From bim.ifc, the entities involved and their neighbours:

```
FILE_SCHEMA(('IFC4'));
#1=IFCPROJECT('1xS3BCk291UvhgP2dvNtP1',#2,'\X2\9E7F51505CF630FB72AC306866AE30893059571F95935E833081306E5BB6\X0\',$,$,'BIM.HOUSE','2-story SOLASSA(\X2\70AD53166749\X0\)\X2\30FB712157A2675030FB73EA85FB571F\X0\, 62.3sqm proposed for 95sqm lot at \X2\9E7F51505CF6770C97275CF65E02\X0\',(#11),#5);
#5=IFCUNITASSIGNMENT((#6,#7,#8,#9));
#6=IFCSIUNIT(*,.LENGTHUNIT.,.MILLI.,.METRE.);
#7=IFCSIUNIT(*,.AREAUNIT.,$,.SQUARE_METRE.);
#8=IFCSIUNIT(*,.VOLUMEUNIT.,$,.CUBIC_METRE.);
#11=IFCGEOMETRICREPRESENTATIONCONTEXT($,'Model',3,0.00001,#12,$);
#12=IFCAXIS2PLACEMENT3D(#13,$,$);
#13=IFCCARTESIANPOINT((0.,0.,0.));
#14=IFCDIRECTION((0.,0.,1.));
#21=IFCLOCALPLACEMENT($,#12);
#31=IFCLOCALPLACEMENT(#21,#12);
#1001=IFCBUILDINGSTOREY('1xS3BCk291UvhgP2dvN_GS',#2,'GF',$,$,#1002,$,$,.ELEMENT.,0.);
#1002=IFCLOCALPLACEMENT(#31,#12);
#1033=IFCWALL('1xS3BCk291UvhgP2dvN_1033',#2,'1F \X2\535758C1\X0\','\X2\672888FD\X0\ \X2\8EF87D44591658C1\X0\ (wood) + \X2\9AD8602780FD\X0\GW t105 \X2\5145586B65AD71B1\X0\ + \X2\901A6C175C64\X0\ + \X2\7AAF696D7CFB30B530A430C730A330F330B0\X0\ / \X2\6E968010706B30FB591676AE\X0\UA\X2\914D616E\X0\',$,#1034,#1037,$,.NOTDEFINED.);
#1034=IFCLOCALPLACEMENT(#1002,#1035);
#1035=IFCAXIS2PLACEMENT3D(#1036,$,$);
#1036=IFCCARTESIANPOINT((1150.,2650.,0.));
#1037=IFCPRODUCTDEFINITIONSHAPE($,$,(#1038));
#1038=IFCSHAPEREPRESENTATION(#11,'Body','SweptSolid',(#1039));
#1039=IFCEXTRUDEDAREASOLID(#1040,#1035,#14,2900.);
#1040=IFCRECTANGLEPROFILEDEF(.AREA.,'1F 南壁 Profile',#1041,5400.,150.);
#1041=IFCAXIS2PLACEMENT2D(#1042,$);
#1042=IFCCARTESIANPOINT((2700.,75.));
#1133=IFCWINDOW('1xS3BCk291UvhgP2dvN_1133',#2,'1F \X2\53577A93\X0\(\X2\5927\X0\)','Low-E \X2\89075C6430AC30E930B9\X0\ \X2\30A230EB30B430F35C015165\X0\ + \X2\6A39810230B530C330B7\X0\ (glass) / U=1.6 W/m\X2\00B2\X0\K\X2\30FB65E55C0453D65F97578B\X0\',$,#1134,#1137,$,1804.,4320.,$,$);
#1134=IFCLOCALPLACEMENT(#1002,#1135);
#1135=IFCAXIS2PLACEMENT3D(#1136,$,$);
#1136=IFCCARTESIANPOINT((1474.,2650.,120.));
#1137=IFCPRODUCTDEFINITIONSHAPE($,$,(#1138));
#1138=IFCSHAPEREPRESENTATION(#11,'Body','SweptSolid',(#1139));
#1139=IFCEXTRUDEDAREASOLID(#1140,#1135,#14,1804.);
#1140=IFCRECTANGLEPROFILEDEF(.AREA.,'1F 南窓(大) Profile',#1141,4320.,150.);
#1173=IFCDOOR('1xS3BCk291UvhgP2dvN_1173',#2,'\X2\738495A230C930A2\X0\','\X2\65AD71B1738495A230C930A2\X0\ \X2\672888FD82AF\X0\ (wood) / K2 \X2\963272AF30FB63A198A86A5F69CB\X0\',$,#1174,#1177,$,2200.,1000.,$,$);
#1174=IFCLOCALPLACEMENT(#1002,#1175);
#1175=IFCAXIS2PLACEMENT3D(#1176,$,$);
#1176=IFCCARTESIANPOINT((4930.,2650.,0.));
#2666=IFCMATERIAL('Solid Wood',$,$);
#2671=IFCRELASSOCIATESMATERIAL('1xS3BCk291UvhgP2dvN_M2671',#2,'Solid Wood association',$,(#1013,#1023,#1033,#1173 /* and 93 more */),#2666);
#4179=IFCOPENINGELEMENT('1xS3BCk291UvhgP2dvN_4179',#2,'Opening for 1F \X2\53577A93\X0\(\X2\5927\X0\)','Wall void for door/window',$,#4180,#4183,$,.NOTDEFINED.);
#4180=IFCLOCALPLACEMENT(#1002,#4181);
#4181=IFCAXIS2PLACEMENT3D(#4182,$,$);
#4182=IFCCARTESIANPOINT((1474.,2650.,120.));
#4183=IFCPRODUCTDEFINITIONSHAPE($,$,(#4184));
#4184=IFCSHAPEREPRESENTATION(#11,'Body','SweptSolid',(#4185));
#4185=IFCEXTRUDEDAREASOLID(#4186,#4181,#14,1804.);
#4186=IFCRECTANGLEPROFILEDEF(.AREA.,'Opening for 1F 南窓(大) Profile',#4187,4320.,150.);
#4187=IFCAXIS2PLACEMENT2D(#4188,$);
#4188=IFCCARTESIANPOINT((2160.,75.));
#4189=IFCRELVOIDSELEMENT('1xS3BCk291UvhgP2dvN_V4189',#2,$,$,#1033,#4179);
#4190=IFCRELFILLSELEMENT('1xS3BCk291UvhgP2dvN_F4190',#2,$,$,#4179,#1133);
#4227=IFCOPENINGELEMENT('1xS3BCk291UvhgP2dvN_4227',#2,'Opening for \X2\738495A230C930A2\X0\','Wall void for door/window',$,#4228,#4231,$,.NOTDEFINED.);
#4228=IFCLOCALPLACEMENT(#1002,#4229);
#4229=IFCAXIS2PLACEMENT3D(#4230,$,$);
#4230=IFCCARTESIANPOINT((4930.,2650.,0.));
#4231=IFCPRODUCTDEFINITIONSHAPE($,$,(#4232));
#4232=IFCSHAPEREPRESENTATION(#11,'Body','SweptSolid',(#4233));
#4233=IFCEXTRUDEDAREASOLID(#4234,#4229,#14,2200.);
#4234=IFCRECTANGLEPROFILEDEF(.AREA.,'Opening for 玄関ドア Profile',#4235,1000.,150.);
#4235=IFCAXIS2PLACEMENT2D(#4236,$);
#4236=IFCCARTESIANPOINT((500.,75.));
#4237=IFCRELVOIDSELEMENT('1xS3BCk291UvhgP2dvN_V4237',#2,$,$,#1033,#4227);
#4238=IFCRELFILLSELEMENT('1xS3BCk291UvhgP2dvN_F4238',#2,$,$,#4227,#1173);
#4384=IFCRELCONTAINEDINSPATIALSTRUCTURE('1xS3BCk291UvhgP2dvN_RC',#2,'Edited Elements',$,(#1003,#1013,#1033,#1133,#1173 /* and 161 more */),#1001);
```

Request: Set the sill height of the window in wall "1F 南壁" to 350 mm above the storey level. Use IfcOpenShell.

```python
import numpy as np
import ifcopenshell
import ifcopenshell.api.geometry
import ifcopenshell.geom
import ifcopenshell.util.element
import ifcopenshell.util.placement
import ifcopenshell.util.shape
import ifcopenshell.util.unit

model = ifcopenshell.open("bim.ifc")
unit_scale = ifcopenshell.util.unit.calculate_unit_scale(model)

window = model.by_guid("1xS3BCk291UvhgP2dvN_1133")
opening = window.FillsVoids[0].RelatingOpeningElement
storey = ifcopenshell.util.element.get_container(window, ifc_class="IfcBuildingStorey")
level = ifcopenshell.util.placement.get_local_placement(storey.ObjectPlacement)[2, 3]

# The opening's origin need not be at the sill, so measure its lowest point.
shape = ifcopenshell.geom.create_shape(ifcopenshell.geom.settings(), opening)
bottom = ifcopenshell.util.shape.get_shape_bottom_elevation(shape, shape.geometry) / unit_scale
dz = level + 0.35 / unit_scale - bottom

shift = np.array([0.0, 0.0, dz])
# The window is not placed relative to its opening, so move both.
for product in (opening, window):
    matrix = ifcopenshell.util.placement.get_local_placement(product.ObjectPlacement)
    matrix[:3, 3] += shift
    ifcopenshell.api.geometry.edit_object_placement(model, product=product, matrix=matrix, is_si=False)

print(f"moved by {dz * unit_scale:+.3f} m")

model.write("bim-out.ifc")
```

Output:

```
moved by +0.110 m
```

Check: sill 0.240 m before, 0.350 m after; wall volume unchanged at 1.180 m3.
